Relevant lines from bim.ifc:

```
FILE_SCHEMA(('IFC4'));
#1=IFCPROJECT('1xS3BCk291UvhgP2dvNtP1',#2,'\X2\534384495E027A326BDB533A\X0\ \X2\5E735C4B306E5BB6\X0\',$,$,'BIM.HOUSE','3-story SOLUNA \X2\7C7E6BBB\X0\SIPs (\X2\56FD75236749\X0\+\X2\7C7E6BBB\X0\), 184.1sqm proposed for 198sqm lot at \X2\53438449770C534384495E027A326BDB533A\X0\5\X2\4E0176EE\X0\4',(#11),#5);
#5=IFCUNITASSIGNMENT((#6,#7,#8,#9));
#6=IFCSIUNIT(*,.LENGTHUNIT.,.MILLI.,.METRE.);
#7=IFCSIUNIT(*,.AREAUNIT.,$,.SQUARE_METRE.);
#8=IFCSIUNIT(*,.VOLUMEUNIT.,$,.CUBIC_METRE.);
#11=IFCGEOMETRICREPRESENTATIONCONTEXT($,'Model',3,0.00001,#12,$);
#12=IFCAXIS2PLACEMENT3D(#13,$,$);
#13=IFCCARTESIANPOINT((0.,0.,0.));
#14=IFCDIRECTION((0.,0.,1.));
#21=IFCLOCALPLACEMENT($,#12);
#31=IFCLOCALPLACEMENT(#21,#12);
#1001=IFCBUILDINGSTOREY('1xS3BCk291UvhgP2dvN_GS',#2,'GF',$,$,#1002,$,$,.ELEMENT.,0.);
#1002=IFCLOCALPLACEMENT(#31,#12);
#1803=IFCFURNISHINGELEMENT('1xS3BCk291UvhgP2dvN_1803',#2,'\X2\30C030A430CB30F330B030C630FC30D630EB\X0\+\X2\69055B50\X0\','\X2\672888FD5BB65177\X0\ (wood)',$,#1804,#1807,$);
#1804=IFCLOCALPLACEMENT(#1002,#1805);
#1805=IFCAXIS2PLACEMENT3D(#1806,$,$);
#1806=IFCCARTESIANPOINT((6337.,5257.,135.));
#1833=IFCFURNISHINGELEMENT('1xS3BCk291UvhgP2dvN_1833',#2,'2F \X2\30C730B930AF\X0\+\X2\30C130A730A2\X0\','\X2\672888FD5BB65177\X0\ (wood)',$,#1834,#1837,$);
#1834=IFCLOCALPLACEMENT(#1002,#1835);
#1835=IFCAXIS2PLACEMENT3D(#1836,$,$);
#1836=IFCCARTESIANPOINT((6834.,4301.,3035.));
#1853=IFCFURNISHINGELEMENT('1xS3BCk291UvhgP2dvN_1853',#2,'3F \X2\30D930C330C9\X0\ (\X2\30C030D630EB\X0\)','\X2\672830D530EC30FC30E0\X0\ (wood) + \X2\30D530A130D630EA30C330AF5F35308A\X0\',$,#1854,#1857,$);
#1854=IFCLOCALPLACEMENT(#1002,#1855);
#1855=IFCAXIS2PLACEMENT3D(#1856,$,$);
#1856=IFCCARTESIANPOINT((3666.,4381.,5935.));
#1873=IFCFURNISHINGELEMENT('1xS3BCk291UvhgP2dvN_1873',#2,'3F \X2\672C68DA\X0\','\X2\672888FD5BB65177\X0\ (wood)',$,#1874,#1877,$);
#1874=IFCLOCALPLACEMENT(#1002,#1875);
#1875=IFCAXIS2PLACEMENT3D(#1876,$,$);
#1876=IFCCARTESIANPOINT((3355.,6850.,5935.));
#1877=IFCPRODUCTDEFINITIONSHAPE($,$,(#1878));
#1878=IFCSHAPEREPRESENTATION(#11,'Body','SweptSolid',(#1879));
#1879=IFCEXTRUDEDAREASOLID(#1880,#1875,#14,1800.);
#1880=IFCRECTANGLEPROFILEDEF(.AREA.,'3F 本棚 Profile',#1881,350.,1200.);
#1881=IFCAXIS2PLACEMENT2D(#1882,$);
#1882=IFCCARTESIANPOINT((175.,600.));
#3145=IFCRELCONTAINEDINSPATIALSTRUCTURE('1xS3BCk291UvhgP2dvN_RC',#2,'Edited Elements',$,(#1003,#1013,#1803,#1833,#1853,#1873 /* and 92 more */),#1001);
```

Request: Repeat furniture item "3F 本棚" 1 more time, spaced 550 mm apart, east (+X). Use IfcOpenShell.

```python
import numpy as np
import ifcopenshell
import ifcopenshell.api.geometry
import ifcopenshell.api.root
import ifcopenshell.util.element
import ifcopenshell.util.placement

model = ifcopenshell.open("bim.ifc")


def reuse_history(source, copy):
    """copy_class also copies each property set's owner history, people and application; keep the originals."""
    for rel in copy.IsDefinedBy:
        if rel.is_a("IfcRelDefinesByProperties") and (history := rel.RelatingPropertyDefinition.OwnerHistory):
            rel.RelatingPropertyDefinition.OwnerHistory = source.OwnerHistory
            ifcopenshell.util.element.remove_deep2(model, history)


source = model.by_guid("1xS3BCk291UvhgP2dvN_1873")
base = ifcopenshell.util.placement.get_local_placement(source.ObjectPlacement)
step = np.array([1.0, 0.0, 0.0]) * 550.0

for i in range(1, 2):
    copy = ifcopenshell.api.root.copy_class(model, product=source)
    copy.Representation = ifcopenshell.util.element.copy_deep(
        model, source.Representation, exclude=["IfcGeometricRepresentationContext", "IfcRepresentationMap"]
    )
    reuse_history(source, copy)
    matrix = base.copy()
    matrix[:3, 3] += i * step
    print("added at", matrix[:3, 3].round(3) + 0.0)
    ifcopenshell.api.geometry.edit_object_placement(model, product=copy, matrix=matrix, is_si=False)

model.write("bim_rev.ifc")
```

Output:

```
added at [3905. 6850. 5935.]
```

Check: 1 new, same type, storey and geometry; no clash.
